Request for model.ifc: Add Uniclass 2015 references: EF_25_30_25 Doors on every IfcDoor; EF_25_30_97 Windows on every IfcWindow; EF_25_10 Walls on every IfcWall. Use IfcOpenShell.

First a look at what the model holds.

```python
import ifcopenshell

model = ifcopenshell.open("model.ifc")
print(model.schema)
print("classifications:", [c.Name for c in model.by_type("IfcClassification")])
for ifc_class in ("IfcDoor", "IfcRoof", "IfcStair", "IfcWall", "IfcWindow"):
    print(ifc_class, len(model.by_type(ifc_class)))
```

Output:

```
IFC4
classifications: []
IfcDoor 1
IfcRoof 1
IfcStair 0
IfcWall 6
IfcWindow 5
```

```python
import ifcopenshell
import ifcopenshell.api.classification

model = ifcopenshell.open("model.ifc")

system = ifcopenshell.api.classification.add_classification(model, classification="Uniclass 2015")

codes = {
    "IfcDoor": ("EF_25_30_25", "Doors"),
    "IfcWindow": ("EF_25_30_97", "Windows"),
    "IfcWall": ("EF_25_10", "Walls"),
}
for ifc_class, (code, name) in codes.items():
    products = model.by_type(ifc_class)
    ifcopenshell.api.classification.add_reference(
        model, products=products, classification=system, identification=code, name=name
    )
    print(code, len(products))

model.write("model_v2.ifc")
```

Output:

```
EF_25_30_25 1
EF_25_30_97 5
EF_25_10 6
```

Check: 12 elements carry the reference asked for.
